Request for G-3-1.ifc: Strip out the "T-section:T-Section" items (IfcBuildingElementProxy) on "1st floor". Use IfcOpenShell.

First a look at what the model holds.

```python
import ifcopenshell
import ifcopenshell.util.element

model = ifcopenshell.open("G-3-1.ifc")
print(model.schema)
storey = next(s for s in model.by_type("IfcBuildingStorey") if s.Name == "1st floor")
proxies = [e for e in ifcopenshell.util.element.get_decomposition(storey) if e.is_a("IfcBuildingElementProxy")]
seen = {}
for e in proxies:
    element_type = ifcopenshell.util.element.get_type(e)
    name = element_type.Name if element_type not in (None, e) else None
    seen[name] = seen.get(name, 0) + 1
for name, count in sorted(seen.items(), key=str):
    print(count, "x", name)
```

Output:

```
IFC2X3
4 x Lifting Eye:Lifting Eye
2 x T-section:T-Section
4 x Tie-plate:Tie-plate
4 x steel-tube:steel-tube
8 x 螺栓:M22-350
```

```python
import ifcopenshell
import ifcopenshell.api.root
import ifcopenshell.util.element

model = ifcopenshell.open("G-3-1.ifc")

storey = next(s for s in model.by_type("IfcBuildingStorey") if s.Name == "1st floor")
proxies = [e for e in ifcopenshell.util.element.get_decomposition(storey) if e.is_a("IfcBuildingElementProxy")]
targets = [e for e in proxies if (t := ifcopenshell.util.element.get_type(e)) not in (None, e) and t.Name == "T-section:T-Section"]

for e in targets:
    ifcopenshell.api.root.remove_product(model, product=e)
print(len(targets), "removed")

model.write("G-3-1_rev.ifc")
```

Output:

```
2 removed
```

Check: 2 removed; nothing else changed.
